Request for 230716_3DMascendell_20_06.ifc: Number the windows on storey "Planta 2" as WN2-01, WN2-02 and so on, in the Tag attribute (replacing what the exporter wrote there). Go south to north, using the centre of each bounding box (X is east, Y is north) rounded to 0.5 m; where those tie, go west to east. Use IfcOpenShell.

First a look at what the model holds.

```python
import ifcopenshell
import ifcopenshell.util.element
import ifcopenshell.util.placement

model = ifcopenshell.open("230716_3DMascendell_20_06.ifc")
print(model.schema)
storey = next(s for s in model.by_type("IfcBuildingStorey") if s.Name == "Planta 2")
windows = [e for e in ifcopenshell.util.element.get_decomposition(storey) if e.is_a("IfcWindow")]
for e in sorted(windows, key=lambda e: e.id()):
    origin = ifcopenshell.util.placement.get_local_placement(e.ObjectPlacement)[:3, 3]
    print(e.id(), e.Tag, e.Name, origin.round(2) + 0.0, sep=" | ")
```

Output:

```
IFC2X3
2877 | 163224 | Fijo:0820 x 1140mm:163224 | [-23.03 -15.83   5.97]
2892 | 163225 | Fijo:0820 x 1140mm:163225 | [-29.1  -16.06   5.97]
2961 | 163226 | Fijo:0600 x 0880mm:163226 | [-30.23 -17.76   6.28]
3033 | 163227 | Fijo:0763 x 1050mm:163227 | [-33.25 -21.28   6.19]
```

```python
import ifcopenshell
import ifcopenshell.geom
import ifcopenshell.util.element
import ifcopenshell.util.shape

model = ifcopenshell.open("230716_3DMascendell_20_06.ifc")
settings = ifcopenshell.geom.settings()
settings.set("use-world-coords", True)


def centre(element):
    shape = ifcopenshell.geom.create_shape(settings, element)
    return ifcopenshell.util.shape.get_bbox_centroid(shape.geometry)


storey = next(s for s in model.by_type("IfcBuildingStorey") if s.Name == "Planta 2")
windows = [e for e in ifcopenshell.util.element.get_decomposition(storey) if e.is_a("IfcWindow")]

# Insertion points can sit at a corner or the storey origin, so sort by the geometry (in metres).
centres = {e: centre(e) for e in windows}
windows.sort(key=lambda e: (round(centres[e][1] / 0.5), centres[e][0]))

for i, e in enumerate(windows, start=1):
    number = f"WN2-{i:02d}"
    e.Tag = number
    print(e.id(), number)

model.write("230716_3DMascendell_20_06_updated.ifc")
```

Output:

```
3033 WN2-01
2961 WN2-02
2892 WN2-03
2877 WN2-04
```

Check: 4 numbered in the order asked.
